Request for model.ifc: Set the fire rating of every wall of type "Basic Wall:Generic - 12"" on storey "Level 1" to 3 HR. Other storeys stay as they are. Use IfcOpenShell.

First a look at what the model holds.

```python
import ifcopenshell
import ifcopenshell.util.element

model = ifcopenshell.open("model.ifc")
print(model.schema)
storey = next(s for s in model.by_type("IfcBuildingStorey") if s.Name == "Level 1")
walls = [e for e in ifcopenshell.util.element.get_decomposition(storey) if e.is_a("IfcWall")]
seen = {}
for e in walls:
    element_type = ifcopenshell.util.element.get_type(e)
    key = (element_type.Name if element_type != e and element_type else None, ifcopenshell.util.element.get_pset(e, "Pset_WallCommon", "FireRating"))
    seen[key] = seen.get(key, 0) + 1
for (name, value), count in sorted(seen.items(), key=str):
    print(count, "x", name, "|", value)
```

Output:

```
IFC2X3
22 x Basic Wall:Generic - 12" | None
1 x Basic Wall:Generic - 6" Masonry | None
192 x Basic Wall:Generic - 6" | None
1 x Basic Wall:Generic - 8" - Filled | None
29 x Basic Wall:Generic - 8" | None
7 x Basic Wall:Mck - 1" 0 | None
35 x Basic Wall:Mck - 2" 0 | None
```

```python
import ifcopenshell
import ifcopenshell.api.pset
import ifcopenshell.util.element

model = ifcopenshell.open("model.ifc")

storey = next(s for s in model.by_type("IfcBuildingStorey") if s.Name == "Level 1")
walls = [e for e in ifcopenshell.util.element.get_decomposition(storey) if e.is_a("IfcWall")]

count = 0
for e in walls:
    element_type = ifcopenshell.util.element.get_type(e)
    if element_type in (None, e) or element_type.Name != 'Basic Wall:Generic - 12"':
        continue
    # add_pset returns the element's existing set when there is one.
    pset = ifcopenshell.api.pset.add_pset(model, product=e, name="Pset_WallCommon")
    ifcopenshell.api.pset.edit_pset(model, pset=pset, properties={"FireRating": "3 HR"})
    count += 1

print(count, "walls updated")

model.write("model_updated.ifc")
```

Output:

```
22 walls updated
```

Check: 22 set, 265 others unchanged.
